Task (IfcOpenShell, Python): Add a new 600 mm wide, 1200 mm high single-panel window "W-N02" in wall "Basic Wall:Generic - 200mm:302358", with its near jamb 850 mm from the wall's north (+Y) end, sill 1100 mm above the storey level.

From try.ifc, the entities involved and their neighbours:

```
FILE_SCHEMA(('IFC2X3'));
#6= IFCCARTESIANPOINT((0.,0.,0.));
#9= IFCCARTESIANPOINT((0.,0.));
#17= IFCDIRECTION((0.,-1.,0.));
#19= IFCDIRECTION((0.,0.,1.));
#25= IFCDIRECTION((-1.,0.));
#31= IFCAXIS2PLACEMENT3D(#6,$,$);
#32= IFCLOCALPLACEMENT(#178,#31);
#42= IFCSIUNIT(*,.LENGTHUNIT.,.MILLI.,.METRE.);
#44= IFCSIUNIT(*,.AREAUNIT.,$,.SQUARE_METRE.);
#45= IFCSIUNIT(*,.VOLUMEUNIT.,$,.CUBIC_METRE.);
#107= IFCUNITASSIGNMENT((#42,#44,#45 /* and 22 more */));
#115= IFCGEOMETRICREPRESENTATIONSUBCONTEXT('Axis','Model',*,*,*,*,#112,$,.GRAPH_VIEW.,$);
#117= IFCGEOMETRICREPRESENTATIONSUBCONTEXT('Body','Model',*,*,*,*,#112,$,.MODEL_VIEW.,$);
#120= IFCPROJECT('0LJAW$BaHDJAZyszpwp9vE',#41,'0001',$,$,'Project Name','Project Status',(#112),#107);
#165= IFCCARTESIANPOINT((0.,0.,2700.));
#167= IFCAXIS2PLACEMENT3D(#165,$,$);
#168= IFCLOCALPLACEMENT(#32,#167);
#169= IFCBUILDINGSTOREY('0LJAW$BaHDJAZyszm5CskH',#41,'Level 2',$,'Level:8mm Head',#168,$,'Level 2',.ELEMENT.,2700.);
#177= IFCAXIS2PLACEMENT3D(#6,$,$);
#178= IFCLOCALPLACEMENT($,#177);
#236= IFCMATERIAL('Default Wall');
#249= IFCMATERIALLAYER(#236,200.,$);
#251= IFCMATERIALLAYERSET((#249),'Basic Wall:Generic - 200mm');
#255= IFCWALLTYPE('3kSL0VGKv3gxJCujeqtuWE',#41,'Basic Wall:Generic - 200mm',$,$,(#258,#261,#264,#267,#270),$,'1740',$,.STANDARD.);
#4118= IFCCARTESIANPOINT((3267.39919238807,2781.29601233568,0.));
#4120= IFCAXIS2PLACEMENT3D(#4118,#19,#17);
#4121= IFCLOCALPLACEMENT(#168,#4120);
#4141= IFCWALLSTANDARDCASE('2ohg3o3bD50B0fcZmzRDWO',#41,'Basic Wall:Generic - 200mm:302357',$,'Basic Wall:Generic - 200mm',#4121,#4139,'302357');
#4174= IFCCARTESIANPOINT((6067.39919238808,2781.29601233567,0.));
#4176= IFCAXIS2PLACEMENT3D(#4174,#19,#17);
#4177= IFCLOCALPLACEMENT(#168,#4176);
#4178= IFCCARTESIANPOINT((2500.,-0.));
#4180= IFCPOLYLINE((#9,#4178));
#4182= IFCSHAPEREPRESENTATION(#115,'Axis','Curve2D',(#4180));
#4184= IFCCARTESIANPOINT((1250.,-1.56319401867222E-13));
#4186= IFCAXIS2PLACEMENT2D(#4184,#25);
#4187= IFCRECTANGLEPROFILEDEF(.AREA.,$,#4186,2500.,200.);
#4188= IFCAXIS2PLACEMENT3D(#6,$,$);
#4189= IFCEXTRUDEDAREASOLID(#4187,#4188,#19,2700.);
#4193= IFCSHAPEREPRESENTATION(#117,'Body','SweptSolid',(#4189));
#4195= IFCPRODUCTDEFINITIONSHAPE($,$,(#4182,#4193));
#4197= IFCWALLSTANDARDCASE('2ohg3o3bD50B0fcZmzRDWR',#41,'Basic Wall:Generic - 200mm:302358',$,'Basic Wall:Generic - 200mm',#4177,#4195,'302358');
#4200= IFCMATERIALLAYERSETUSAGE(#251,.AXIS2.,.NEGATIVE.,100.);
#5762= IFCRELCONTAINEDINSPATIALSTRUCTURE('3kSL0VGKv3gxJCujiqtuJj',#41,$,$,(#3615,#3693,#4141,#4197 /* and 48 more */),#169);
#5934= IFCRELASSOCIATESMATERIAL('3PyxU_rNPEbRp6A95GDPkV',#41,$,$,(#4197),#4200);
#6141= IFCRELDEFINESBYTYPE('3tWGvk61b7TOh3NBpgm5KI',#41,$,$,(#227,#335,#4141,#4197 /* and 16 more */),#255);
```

```python
import numpy as np
import ifcopenshell
import ifcopenshell.api.feature
import ifcopenshell.api.geometry
import ifcopenshell.api.root
import ifcopenshell.api.spatial
import ifcopenshell.api.type
import ifcopenshell.geom
import ifcopenshell.util.element
import ifcopenshell.util.placement
import ifcopenshell.util.representation
import ifcopenshell.util.shape
import ifcopenshell.util.unit

model = ifcopenshell.open("try.ifc")
unit_scale = ifcopenshell.util.unit.calculate_unit_scale(model)
settings = ifcopenshell.geom.settings()


def volume(element):
    """Net volume in cubic metres, openings subtracted."""
    shape = ifcopenshell.geom.create_shape(settings, element)
    return ifcopenshell.util.shape.get_volume(shape.geometry)


wall = model.by_id(4197)
storey = ifcopenshell.util.element.get_container(wall, ifc_class="IfcBuildingStorey")
context = ifcopenshell.util.representation.get_context(model, "Model", "Body", "MODEL_VIEW")
before = volume(wall)

width, height, from_end, sill = 0.6, 1.2, 0.85, 1.1  # metres

# The wall runs along its own X axis, and the end named is its -X end.
wall_shape = ifcopenshell.geom.create_shape(settings, wall)
x, y, z = ifcopenshell.util.shape.get_vertices(wall_shape.geometry).T
start = x.min() + from_end
face, thickness = float(y.min()), float(y.max() - y.min())
wall_matrix = ifcopenshell.util.placement.get_local_placement(wall.ObjectPlacement)
level = ifcopenshell.util.placement.get_local_placement(storey.ObjectPlacement)[2, 3]


def in_wall(x, y):
    """Placement at x, y metres in the wall's axes, at sill height."""
    matrix = wall_matrix.copy()
    matrix[:, 3] = wall_matrix @ np.array([x / unit_scale, y / unit_scale, 0.0, 1.0])
    matrix[2, 3] = level + sill / unit_scale
    return matrix


# Opening: a box that overshoots both wall faces by 50 mm.
opening = ifcopenshell.api.root.create_entity(model, ifc_class="IfcOpeningElement")
box = ifcopenshell.api.geometry.add_wall_representation(
    model, context=context, length=width, height=height, thickness=thickness + 0.1
)
ifcopenshell.api.geometry.assign_representation(model, product=opening, representation=box)
ifcopenshell.api.geometry.edit_object_placement(model, product=opening, matrix=in_wall(start, face - 0.05), is_si=False)
ifcopenshell.api.feature.add_feature(model, feature=opening, element=wall)

window = ifcopenshell.api.root.create_entity(model, ifc_class="IfcWindow", name="W-N02")
window.OverallWidth, window.OverallHeight = width / unit_scale, height / unit_scale
body = ifcopenshell.api.geometry.add_window_representation(
    model,
    context=context,
    overall_width=window.OverallWidth,
    overall_height=window.OverallHeight,
    partition_type="SINGLE_PANEL",
)
ifcopenshell.api.geometry.assign_representation(model, product=window, representation=body)
ifcopenshell.api.spatial.assign_container(model, products=[window], relating_structure=storey)
fills = ifcopenshell.api.feature.add_filling(model, opening=opening, element=window)
fills.OwnerHistory = window.OwnerHistory  # required in IFC2X3

# IFC2X3 keeps the operation on the window style.
style = ifcopenshell.api.root.create_entity(model, ifc_class="IfcWindowStyle", name="W-N02")
style.OperationType, style.ConstructionType = "SINGLE_PANEL", "NOTDEFINED"
style.ParameterTakesPrecedence = style.Sizeable = False
ifcopenshell.api.type.assign_type(model, related_objects=[window], relating_type=style)

# Centre the window in the wall's thickness.
ifcopenshell.api.geometry.edit_object_placement(model, product=window, matrix=in_wall(start, face), is_si=False)
window_shape = ifcopenshell.geom.create_shape(settings, window)
depth = ifcopenshell.util.shape.get_vertices(window_shape.geometry)[:, 1]
offset = face + thickness / 2 - (depth.min() + depth.max()) / 2
ifcopenshell.api.geometry.edit_object_placement(model, product=window, matrix=in_wall(start, offset), is_si=False)

after = volume(wall)

print(f"wall volume {before:.3f} -> {after:.3f} m3")

model.write("try_v2.ifc")
```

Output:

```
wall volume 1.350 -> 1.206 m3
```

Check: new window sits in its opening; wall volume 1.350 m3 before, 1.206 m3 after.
